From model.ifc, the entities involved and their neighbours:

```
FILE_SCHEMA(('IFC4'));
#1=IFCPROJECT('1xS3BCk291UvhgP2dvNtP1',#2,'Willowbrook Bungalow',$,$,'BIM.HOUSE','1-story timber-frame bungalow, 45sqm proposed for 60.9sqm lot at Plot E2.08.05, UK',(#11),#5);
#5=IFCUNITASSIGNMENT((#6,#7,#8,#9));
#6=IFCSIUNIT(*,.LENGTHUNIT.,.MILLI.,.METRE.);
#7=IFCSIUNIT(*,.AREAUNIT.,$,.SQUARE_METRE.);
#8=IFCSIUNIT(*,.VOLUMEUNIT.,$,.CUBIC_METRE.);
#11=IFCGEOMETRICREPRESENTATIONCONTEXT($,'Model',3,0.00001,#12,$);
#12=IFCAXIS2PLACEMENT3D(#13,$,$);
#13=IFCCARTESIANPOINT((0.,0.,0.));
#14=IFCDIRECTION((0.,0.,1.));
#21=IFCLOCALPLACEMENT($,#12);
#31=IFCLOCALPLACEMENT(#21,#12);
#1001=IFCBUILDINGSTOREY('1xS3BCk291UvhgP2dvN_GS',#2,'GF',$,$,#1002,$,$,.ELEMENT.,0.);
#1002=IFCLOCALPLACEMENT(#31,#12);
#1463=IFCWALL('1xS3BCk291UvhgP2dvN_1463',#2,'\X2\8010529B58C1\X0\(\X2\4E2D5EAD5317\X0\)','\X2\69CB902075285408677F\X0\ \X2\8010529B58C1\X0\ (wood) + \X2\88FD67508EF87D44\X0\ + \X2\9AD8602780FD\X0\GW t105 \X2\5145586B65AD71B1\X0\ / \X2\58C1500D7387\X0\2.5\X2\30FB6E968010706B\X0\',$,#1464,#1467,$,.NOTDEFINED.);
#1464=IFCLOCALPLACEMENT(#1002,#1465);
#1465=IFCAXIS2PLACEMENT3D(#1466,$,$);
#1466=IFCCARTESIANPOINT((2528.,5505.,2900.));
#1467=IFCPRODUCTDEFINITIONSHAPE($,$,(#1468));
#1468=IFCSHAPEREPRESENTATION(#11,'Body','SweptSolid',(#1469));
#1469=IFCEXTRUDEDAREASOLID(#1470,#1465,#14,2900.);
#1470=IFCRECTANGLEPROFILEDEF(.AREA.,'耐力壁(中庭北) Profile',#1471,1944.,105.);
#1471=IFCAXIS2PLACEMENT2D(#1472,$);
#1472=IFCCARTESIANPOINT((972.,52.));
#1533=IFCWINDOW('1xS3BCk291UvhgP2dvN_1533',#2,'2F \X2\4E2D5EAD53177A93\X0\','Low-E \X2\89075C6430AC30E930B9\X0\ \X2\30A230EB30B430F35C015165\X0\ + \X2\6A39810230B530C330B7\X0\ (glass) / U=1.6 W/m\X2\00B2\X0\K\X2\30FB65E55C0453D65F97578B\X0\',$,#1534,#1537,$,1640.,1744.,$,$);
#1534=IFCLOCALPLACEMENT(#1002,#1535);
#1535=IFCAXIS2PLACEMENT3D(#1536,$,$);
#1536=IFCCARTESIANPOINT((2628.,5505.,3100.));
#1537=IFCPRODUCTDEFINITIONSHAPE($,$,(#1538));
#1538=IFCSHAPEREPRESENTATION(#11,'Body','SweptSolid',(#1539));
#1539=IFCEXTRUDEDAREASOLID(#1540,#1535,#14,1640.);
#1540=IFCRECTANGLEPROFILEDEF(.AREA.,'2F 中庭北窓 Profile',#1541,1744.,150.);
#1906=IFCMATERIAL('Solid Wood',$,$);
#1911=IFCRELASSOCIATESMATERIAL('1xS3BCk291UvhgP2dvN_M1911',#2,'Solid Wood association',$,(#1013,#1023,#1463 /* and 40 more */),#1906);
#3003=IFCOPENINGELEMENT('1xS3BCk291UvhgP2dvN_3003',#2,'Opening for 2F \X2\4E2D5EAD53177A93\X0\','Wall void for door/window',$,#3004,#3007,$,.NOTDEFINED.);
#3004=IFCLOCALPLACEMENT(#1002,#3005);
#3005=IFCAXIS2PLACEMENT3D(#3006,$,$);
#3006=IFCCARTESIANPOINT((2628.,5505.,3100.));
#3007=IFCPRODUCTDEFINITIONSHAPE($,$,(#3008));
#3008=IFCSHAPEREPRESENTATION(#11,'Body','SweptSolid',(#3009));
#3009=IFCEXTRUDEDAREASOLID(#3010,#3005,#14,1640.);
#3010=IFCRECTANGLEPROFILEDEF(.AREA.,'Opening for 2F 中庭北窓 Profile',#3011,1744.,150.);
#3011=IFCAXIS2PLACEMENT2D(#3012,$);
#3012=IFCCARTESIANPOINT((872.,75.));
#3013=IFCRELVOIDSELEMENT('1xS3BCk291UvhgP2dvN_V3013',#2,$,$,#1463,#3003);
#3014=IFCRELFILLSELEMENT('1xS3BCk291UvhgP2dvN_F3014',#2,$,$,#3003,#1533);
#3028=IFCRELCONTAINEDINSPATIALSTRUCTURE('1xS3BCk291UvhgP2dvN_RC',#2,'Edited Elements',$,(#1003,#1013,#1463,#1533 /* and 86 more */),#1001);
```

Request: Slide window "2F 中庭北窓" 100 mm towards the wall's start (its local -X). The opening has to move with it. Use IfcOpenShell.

```python
import ifcopenshell
import ifcopenshell.api.geometry
import ifcopenshell.util.placement
import ifcopenshell.util.unit

model = ifcopenshell.open("model.ifc")
unit_scale = ifcopenshell.util.unit.calculate_unit_scale(model)

window = model.by_guid("1xS3BCk291UvhgP2dvN_1533")
opening = window.FillsVoids[0].RelatingOpeningElement
wall = opening.VoidsElements[0].RelatingBuildingElement

wall_matrix = ifcopenshell.util.placement.get_local_placement(wall.ObjectPlacement)
shift = wall_matrix[:3, 0] * -0.1 / unit_scale
before = ifcopenshell.util.placement.get_local_placement(window.ObjectPlacement)[:3, 3].copy()

# The window is not placed relative to its opening, so move both.
for product in (opening, window):
    matrix = ifcopenshell.util.placement.get_local_placement(product.ObjectPlacement)
    matrix[:3, 3] += shift
    ifcopenshell.api.geometry.edit_object_placement(model, product=product, matrix=matrix, is_si=False)

after = ifcopenshell.util.placement.get_local_placement(window.ObjectPlacement)[:3, 3]
print("window moved by", (after - before).round(3) + 0.0)

model.write("model_updated.ifc")
```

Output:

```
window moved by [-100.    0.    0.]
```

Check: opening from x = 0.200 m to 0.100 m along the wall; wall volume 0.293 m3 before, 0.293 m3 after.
